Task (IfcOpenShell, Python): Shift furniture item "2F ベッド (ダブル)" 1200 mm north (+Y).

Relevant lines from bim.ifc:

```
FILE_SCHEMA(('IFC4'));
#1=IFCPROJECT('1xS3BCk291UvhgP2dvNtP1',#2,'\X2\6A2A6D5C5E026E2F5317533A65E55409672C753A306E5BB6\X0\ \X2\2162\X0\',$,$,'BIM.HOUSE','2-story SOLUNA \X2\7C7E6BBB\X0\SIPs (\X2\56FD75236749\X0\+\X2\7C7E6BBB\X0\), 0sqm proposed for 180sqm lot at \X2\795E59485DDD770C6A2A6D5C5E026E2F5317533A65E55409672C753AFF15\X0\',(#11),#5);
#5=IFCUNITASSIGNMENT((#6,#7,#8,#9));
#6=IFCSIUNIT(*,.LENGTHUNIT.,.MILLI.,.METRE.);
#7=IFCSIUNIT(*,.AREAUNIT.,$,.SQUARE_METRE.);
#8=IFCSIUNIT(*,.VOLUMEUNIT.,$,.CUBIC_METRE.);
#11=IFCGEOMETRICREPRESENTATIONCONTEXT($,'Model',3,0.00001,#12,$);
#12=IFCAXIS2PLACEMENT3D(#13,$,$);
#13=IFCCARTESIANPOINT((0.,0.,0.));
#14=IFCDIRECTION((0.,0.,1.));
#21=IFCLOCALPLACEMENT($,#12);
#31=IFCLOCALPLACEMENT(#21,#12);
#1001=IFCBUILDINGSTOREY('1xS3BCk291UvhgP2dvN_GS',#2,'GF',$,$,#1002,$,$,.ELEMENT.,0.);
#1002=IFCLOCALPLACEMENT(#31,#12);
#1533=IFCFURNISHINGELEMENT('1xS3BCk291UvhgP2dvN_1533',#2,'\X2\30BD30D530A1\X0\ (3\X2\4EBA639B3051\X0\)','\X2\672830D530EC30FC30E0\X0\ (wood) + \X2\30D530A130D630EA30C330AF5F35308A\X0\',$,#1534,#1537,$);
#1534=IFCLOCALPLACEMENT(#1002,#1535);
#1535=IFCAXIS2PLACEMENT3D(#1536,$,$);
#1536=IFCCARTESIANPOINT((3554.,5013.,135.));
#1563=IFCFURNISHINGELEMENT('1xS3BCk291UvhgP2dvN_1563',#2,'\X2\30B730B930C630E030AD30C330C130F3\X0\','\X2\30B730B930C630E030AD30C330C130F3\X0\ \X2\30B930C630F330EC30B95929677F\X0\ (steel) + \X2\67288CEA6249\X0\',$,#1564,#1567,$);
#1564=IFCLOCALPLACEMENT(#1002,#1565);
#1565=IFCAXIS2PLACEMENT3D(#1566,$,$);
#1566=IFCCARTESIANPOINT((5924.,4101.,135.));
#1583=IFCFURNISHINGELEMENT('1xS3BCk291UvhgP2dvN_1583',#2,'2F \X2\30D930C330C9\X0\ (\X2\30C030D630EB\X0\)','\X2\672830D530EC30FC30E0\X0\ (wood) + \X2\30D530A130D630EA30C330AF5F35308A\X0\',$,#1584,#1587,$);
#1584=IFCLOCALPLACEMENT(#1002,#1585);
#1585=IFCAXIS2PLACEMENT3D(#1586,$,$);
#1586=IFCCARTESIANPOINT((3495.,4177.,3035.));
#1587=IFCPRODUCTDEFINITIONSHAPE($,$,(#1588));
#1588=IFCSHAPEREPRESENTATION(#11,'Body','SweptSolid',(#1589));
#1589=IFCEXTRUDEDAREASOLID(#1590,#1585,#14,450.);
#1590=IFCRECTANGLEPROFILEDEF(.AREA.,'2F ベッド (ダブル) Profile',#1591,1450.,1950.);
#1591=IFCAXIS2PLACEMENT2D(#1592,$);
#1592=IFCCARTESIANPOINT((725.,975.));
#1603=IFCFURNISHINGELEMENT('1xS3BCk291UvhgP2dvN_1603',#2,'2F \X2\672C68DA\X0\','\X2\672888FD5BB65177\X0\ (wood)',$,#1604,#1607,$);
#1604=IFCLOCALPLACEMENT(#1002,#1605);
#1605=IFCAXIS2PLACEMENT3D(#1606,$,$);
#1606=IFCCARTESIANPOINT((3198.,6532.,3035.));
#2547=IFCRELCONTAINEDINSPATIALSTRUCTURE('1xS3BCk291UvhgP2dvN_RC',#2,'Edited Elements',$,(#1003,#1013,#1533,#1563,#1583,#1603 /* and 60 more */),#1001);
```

```python
import ifcopenshell
import ifcopenshell.api.geometry
import ifcopenshell.util.placement
import ifcopenshell.util.unit

model = ifcopenshell.open("bim.ifc")
unit_scale = ifcopenshell.util.unit.calculate_unit_scale(model)

item = model.by_guid("1xS3BCk291UvhgP2dvN_1583")
matrix = ifcopenshell.util.placement.get_local_placement(item.ObjectPlacement)
matrix[1, 3] += 1.2 / unit_scale
ifcopenshell.api.geometry.edit_object_placement(model, product=item, matrix=matrix, is_si=False)

print(ifcopenshell.util.placement.get_local_placement(item.ObjectPlacement).round(3) + 0.0)

model.write("bim_updated.ifc")
```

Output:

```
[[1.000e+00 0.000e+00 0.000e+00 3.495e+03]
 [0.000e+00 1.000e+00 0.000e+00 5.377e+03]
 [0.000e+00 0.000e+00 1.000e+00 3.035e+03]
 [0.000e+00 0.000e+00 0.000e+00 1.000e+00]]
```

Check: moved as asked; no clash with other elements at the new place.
